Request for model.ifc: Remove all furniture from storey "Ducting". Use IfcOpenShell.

First a look at what the model holds.

```python
import ifcopenshell
import ifcopenshell.util.element

model = ifcopenshell.open("model.ifc")
print(model.schema)
storey = next(s for s in model.by_type("IfcBuildingStorey") if s.Name == "Ducting")
furniture = [e for e in ifcopenshell.util.element.get_decomposition(storey) if e.is_a("IfcFurnishingElement")]
seen = {}
for e in furniture:
    element_type = ifcopenshell.util.element.get_type(e)
    name = element_type.Name if element_type not in (None, e) else None
    seen[name] = seen.get(name, 0) + 1
for name, count in sorted(seen.items(), key=str):
    print(count, "x", name)
```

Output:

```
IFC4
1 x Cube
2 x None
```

```python
import ifcopenshell
import ifcopenshell.api.root
import ifcopenshell.util.element

model = ifcopenshell.open("model.ifc")

storey = next(s for s in model.by_type("IfcBuildingStorey") if s.Name == "Ducting")
furniture = [e for e in ifcopenshell.util.element.get_decomposition(storey) if e.is_a("IfcFurnishingElement")]

for e in furniture:
    ifcopenshell.api.root.remove_product(model, product=e)
print(len(furniture), "removed")

model.write("model_edited.ifc")
```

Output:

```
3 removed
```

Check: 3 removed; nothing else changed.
